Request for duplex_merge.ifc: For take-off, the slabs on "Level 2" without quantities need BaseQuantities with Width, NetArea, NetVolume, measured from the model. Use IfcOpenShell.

First a look at what the model holds.

```python
import ifcopenshell
import ifcopenshell.util.element
import ifcopenshell.util.unit

model = ifcopenshell.open("duplex_merge.ifc")
print(model.schema)
for unit_type in ("LENGTHUNIT", "AREAUNIT", "VOLUMEUNIT"):
    print(unit_type, ifcopenshell.util.unit.calculate_unit_scale(model, unit_type))
storey = next(s for s in model.by_type("IfcBuildingStorey") if s.Name == "Level 2")
slabs = [e for e in ifcopenshell.util.element.get_decomposition(storey) if e.is_a("IfcSlab")]
for e in sorted(slabs, key=lambda e: e.id()):
    print(e.id(), e.is_a(), e.Name, list(ifcopenshell.util.element.get_psets(e, qtos_only=True)), sep=" | ")
```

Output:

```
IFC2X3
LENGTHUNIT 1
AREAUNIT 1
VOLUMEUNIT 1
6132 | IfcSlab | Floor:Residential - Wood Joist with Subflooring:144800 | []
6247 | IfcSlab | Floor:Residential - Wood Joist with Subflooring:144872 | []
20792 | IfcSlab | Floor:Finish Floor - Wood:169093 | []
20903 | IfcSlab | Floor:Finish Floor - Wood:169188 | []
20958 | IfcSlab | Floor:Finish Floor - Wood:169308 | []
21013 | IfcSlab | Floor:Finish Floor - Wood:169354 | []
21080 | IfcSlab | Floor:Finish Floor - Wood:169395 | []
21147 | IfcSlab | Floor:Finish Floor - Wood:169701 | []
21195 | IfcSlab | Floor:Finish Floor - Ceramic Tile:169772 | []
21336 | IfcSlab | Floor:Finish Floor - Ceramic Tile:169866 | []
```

```python
import ifcopenshell
import ifcopenshell.api.pset
import ifcopenshell.geom
import ifcopenshell.util.element
import ifcopenshell.util.shape
import ifcopenshell.util.unit

model = ifcopenshell.open("duplex_merge.ifc")
unit_scale = ifcopenshell.util.unit.calculate_unit_scale(model)
area_scale = ifcopenshell.util.unit.calculate_unit_scale(model, "AREAUNIT")
volume_scale = ifcopenshell.util.unit.calculate_unit_scale(model, "VOLUMEUNIT")
settings = ifcopenshell.geom.settings()

storey = next(s for s in model.by_type("IfcBuildingStorey") if s.Name == "Level 2")
slabs = [e for e in ifcopenshell.util.element.get_decomposition(storey) if e.is_a("IfcSlab")]

for e in sorted(slabs, key=lambda e: e.id()):
    if ifcopenshell.util.element.get_psets(e, qtos_only=True, should_inherit=False):
        continue
    # Geometry comes back in metres, in the element's own axes.
    shape = ifcopenshell.geom.create_shape(settings, e)
    values = {
        "Width": ifcopenshell.util.shape.get_z(shape.geometry) / unit_scale,
        "NetArea": ifcopenshell.util.shape.get_footprint_area(shape.geometry) / area_scale,
        "NetVolume": ifcopenshell.util.shape.get_volume(shape.geometry) / volume_scale,
    }
    qto = ifcopenshell.api.pset.add_qto(model, product=e, name="BaseQuantities")
    ifcopenshell.api.pset.edit_qto(model, qto=qto, properties=values)
    print(e.id(), {k: round(v, 3) for k, v in values.items()})

model.write("duplex_merge_rev.ifc")
```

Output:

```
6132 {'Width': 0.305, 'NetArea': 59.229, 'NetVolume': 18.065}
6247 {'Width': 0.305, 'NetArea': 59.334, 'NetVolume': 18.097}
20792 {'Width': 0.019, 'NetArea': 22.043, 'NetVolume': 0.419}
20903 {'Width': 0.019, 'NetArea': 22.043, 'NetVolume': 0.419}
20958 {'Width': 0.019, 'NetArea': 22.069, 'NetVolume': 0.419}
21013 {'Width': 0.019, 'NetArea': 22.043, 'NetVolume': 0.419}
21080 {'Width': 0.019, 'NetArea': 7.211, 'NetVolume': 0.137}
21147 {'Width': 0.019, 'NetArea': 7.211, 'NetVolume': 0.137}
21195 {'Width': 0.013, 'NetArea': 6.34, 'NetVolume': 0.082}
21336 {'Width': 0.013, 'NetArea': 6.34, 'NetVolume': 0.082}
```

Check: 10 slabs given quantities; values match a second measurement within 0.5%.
